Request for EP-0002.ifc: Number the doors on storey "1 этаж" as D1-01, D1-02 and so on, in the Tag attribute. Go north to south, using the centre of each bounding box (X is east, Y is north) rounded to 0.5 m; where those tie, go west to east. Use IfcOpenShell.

First a look at what the model holds.

```python
import ifcopenshell
import ifcopenshell.util.element
import ifcopenshell.util.placement

model = ifcopenshell.open("EP-0002.ifc")
print(model.schema)
storey = next(s for s in model.by_type("IfcBuildingStorey") if s.Name == "1 этаж")
doors = [e for e in ifcopenshell.util.element.get_decomposition(storey) if e.is_a("IfcDoor")]
for e in sorted(doors, key=lambda e: e.id()):
    origin = ifcopenshell.util.placement.get_local_placement(e.ObjectPlacement)[:3, 3]
    print(e.id(), e.Tag, e.Name, origin.round(2) + 0.0, sep=" | ")
```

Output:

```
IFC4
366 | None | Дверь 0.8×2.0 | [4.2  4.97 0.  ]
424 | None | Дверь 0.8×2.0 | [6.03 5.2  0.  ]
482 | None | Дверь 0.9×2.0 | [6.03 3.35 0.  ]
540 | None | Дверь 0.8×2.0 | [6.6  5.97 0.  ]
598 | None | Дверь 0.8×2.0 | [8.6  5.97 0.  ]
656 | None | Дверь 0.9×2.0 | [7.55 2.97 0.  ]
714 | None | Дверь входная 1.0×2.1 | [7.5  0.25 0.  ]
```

```python
import ifcopenshell
import ifcopenshell.geom
import ifcopenshell.util.element
import ifcopenshell.util.shape

model = ifcopenshell.open("EP-0002.ifc")
settings = ifcopenshell.geom.settings()
settings.set("use-world-coords", True)


def centre(element):
    shape = ifcopenshell.geom.create_shape(settings, element)
    return ifcopenshell.util.shape.get_bbox_centroid(shape.geometry)


storey = next(s for s in model.by_type("IfcBuildingStorey") if s.Name == "1 этаж")
doors = [e for e in ifcopenshell.util.element.get_decomposition(storey) if e.is_a("IfcDoor")]

# Insertion points can sit at a corner or the storey origin, so sort by the geometry (in metres).
centres = {e: centre(e) for e in doors}
doors.sort(key=lambda e: (-round(centres[e][1] / 0.5), centres[e][0]))

for i, e in enumerate(doors, start=1):
    number = f"D1-{i:02d}"
    e.Tag = number
    print(e.id(), number)

model.write("EP-0002_v2.ifc")
```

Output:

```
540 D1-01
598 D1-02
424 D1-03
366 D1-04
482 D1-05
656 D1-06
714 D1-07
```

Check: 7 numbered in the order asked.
